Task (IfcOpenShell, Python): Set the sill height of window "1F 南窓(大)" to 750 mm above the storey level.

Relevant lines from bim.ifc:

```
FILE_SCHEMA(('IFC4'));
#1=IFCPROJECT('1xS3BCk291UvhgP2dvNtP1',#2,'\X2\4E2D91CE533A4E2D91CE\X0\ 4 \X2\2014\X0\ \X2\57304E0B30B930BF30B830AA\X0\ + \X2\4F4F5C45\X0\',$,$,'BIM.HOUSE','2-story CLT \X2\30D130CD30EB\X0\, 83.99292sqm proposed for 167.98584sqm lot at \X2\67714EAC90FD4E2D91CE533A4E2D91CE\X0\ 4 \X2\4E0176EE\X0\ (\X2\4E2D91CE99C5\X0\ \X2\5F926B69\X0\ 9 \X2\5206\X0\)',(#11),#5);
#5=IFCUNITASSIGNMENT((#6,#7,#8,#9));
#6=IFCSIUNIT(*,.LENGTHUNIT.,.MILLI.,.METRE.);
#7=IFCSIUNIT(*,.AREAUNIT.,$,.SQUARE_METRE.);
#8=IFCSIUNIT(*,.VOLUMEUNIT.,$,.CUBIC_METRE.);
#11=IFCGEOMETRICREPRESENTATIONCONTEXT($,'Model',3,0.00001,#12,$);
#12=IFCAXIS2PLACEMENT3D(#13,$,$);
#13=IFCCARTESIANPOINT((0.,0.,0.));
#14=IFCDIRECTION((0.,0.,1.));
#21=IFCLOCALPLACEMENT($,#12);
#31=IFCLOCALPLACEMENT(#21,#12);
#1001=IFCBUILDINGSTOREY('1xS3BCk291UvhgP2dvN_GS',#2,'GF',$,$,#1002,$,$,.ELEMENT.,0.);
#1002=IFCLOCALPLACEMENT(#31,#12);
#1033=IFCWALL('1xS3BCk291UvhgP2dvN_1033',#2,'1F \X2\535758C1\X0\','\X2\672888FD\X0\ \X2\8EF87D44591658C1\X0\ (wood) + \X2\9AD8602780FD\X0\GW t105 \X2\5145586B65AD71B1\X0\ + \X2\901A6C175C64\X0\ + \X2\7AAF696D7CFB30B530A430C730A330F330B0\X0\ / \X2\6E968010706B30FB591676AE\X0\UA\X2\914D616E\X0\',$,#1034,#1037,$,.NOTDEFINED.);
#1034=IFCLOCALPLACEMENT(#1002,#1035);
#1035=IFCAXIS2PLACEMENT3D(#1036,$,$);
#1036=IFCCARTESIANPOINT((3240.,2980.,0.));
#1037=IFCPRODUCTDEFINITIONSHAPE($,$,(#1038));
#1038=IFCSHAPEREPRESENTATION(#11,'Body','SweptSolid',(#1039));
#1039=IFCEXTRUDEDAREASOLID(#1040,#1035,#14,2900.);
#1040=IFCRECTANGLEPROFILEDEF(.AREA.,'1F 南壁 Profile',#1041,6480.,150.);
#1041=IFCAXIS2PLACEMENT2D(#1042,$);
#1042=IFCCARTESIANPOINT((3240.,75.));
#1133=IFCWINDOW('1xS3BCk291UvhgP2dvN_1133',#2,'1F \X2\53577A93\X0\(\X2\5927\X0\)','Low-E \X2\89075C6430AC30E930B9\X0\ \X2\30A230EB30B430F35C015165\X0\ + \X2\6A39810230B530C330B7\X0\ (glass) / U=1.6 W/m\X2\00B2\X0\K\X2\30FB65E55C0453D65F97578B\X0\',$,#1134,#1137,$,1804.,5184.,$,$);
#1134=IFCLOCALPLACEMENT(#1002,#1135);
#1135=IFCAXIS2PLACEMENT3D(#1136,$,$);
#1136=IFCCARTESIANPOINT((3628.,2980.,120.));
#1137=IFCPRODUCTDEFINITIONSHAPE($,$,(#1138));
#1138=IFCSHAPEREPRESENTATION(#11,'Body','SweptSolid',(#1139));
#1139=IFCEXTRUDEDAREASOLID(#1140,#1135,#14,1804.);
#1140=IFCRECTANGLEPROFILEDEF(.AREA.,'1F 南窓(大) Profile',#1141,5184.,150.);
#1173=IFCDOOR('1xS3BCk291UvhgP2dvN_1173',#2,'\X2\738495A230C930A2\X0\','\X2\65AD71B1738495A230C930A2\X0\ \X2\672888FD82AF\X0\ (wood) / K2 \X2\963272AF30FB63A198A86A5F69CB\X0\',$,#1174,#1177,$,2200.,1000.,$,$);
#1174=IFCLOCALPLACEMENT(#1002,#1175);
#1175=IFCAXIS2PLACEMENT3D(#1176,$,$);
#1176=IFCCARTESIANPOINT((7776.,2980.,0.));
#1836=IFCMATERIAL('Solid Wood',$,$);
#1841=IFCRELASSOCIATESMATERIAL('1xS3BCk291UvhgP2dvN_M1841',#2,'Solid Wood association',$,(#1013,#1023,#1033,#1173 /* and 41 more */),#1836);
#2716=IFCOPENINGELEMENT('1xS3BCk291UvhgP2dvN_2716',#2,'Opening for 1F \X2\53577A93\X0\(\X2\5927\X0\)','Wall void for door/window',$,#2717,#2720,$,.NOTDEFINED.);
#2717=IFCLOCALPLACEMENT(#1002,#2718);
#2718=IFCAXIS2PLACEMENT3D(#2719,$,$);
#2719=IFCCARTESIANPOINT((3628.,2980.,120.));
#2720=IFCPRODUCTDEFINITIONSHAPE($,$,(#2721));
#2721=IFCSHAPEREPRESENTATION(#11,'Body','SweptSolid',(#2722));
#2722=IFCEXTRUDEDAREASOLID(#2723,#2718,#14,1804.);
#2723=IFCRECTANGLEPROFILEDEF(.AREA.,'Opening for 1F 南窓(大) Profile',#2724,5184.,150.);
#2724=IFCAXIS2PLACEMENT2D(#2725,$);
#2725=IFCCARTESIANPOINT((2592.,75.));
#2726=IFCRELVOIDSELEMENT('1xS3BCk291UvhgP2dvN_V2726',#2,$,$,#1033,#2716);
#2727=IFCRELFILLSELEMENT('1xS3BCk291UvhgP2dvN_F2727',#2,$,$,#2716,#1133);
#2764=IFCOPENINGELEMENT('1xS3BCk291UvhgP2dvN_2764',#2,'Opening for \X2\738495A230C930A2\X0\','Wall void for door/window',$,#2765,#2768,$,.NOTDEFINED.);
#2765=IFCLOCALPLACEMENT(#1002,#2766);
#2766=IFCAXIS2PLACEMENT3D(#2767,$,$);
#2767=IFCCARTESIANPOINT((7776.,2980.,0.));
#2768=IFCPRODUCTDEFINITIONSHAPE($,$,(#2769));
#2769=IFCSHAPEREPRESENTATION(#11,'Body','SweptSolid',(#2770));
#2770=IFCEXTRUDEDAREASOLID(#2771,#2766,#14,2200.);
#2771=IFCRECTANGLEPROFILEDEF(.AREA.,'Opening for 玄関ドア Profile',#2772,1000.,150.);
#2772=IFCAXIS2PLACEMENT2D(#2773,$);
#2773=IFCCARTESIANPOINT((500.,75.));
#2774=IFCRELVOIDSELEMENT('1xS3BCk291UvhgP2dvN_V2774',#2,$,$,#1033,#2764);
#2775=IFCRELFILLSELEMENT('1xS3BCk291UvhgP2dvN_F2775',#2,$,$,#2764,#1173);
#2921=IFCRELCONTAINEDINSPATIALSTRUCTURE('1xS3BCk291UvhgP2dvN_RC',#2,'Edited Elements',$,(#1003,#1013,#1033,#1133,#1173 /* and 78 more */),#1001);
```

```python
import numpy as np
import ifcopenshell
import ifcopenshell.api.geometry
import ifcopenshell.geom
import ifcopenshell.util.element
import ifcopenshell.util.placement
import ifcopenshell.util.shape
import ifcopenshell.util.unit

model = ifcopenshell.open("bim.ifc")
unit_scale = ifcopenshell.util.unit.calculate_unit_scale(model)

window = model.by_id(1133)
opening = window.FillsVoids[0].RelatingOpeningElement
storey = ifcopenshell.util.element.get_container(window, ifc_class="IfcBuildingStorey")
level = ifcopenshell.util.placement.get_local_placement(storey.ObjectPlacement)[2, 3]

# The opening's origin need not be at the sill, so measure its lowest point.
shape = ifcopenshell.geom.create_shape(ifcopenshell.geom.settings(), opening)
bottom = ifcopenshell.util.shape.get_shape_bottom_elevation(shape, shape.geometry) / unit_scale
dz = level + 750.0 - bottom

shift = np.array([0.0, 0.0, dz])
# The window is not placed relative to its opening, so move both.
for product in (opening, window):
    matrix = ifcopenshell.util.placement.get_local_placement(product.ObjectPlacement)
    matrix[:3, 3] += shift
    ifcopenshell.api.geometry.edit_object_placement(model, product=product, matrix=matrix, is_si=False)

print(f"moved by {dz * unit_scale:+.3f} m")

model.write("bim-out.ifc")
```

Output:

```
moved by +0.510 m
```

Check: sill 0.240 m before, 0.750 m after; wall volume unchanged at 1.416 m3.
